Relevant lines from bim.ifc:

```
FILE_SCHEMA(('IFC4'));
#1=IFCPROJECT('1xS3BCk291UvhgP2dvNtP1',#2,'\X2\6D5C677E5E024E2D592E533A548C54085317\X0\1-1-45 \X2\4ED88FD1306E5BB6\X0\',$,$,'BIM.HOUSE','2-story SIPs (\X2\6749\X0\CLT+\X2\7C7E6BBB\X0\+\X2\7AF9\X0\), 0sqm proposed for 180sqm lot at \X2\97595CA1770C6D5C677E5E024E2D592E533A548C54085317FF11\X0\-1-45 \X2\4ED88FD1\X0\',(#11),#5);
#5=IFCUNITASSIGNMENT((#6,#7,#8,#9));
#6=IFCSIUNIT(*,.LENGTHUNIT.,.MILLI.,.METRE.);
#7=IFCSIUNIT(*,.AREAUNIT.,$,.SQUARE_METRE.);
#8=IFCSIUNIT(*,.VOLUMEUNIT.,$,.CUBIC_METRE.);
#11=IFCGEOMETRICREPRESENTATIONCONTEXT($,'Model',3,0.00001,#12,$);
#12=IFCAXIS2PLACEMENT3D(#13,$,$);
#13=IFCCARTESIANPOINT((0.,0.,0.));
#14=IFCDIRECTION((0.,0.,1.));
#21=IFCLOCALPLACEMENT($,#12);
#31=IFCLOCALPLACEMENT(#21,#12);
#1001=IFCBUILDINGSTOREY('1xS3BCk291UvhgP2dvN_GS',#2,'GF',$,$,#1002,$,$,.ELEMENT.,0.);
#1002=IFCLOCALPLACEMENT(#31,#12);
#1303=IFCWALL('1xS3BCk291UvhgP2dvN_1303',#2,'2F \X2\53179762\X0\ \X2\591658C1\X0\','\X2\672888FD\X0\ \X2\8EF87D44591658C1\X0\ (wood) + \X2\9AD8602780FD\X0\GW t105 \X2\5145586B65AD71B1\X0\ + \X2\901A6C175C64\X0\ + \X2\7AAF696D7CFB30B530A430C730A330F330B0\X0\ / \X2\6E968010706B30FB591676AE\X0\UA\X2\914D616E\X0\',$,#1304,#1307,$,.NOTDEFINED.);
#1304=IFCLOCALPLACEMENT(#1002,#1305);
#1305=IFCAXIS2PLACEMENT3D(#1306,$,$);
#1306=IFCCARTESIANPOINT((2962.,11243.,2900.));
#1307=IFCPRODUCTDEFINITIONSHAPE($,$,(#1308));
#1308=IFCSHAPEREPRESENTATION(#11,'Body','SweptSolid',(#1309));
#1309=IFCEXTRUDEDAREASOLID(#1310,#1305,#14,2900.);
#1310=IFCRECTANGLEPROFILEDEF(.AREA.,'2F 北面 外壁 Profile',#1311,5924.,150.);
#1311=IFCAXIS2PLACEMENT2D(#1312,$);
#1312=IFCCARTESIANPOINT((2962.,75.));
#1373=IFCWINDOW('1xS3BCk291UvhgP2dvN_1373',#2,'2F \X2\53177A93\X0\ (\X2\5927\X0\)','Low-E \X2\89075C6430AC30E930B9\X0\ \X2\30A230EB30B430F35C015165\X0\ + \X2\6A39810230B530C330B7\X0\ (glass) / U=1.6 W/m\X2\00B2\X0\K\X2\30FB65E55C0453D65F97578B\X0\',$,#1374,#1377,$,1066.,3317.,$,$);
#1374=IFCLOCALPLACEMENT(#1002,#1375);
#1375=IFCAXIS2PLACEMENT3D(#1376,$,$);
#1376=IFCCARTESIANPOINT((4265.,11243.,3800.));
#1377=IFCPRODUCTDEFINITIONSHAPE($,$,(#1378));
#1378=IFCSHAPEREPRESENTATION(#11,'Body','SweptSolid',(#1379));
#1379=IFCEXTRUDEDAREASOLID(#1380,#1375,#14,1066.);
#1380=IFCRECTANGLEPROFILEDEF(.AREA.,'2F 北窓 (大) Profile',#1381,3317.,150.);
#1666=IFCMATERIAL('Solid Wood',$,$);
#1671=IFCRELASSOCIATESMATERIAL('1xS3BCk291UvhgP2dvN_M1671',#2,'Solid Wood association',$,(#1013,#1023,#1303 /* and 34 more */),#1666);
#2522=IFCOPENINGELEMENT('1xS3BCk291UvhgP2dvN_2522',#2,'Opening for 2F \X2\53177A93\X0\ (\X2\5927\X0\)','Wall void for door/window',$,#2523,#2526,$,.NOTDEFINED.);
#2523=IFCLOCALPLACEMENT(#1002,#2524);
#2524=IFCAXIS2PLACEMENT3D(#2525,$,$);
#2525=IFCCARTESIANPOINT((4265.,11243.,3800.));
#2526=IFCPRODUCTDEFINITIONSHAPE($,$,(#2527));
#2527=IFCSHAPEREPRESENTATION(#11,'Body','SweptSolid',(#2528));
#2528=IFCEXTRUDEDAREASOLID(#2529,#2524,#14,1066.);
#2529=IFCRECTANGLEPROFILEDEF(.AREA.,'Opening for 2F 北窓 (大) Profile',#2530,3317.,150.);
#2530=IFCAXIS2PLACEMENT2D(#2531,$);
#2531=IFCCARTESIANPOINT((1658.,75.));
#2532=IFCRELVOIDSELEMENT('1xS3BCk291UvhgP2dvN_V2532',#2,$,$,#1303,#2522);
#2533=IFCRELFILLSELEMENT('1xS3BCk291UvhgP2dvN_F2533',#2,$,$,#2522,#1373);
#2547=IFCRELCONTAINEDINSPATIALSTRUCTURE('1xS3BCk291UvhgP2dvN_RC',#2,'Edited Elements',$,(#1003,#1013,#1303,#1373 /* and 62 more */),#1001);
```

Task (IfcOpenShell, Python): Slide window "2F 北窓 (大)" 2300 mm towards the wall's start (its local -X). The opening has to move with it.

```python
import ifcopenshell
import ifcopenshell.api.geometry
import ifcopenshell.util.placement
import ifcopenshell.util.unit

model = ifcopenshell.open("bim.ifc")
unit_scale = ifcopenshell.util.unit.calculate_unit_scale(model)

window = model.by_guid("1xS3BCk291UvhgP2dvN_1373")
opening = window.FillsVoids[0].RelatingOpeningElement
wall = opening.VoidsElements[0].RelatingBuildingElement

wall_matrix = ifcopenshell.util.placement.get_local_placement(wall.ObjectPlacement)
shift = wall_matrix[:3, 0] * -2.3 / unit_scale
before = ifcopenshell.util.placement.get_local_placement(window.ObjectPlacement)[:3, 3].copy()

# The window is not placed relative to its opening, so move both.
for product in (opening, window):
    matrix = ifcopenshell.util.placement.get_local_placement(product.ObjectPlacement)
    matrix[:3, 3] += shift
    ifcopenshell.api.geometry.edit_object_placement(model, product=product, matrix=matrix, is_si=False)

after = ifcopenshell.util.placement.get_local_placement(window.ObjectPlacement)[:3, 3]
print("window moved by", (after - before).round(3) + 0.0)

model.write("bim_rev.ifc")
```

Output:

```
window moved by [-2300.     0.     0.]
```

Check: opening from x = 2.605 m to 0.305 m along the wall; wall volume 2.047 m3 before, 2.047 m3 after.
